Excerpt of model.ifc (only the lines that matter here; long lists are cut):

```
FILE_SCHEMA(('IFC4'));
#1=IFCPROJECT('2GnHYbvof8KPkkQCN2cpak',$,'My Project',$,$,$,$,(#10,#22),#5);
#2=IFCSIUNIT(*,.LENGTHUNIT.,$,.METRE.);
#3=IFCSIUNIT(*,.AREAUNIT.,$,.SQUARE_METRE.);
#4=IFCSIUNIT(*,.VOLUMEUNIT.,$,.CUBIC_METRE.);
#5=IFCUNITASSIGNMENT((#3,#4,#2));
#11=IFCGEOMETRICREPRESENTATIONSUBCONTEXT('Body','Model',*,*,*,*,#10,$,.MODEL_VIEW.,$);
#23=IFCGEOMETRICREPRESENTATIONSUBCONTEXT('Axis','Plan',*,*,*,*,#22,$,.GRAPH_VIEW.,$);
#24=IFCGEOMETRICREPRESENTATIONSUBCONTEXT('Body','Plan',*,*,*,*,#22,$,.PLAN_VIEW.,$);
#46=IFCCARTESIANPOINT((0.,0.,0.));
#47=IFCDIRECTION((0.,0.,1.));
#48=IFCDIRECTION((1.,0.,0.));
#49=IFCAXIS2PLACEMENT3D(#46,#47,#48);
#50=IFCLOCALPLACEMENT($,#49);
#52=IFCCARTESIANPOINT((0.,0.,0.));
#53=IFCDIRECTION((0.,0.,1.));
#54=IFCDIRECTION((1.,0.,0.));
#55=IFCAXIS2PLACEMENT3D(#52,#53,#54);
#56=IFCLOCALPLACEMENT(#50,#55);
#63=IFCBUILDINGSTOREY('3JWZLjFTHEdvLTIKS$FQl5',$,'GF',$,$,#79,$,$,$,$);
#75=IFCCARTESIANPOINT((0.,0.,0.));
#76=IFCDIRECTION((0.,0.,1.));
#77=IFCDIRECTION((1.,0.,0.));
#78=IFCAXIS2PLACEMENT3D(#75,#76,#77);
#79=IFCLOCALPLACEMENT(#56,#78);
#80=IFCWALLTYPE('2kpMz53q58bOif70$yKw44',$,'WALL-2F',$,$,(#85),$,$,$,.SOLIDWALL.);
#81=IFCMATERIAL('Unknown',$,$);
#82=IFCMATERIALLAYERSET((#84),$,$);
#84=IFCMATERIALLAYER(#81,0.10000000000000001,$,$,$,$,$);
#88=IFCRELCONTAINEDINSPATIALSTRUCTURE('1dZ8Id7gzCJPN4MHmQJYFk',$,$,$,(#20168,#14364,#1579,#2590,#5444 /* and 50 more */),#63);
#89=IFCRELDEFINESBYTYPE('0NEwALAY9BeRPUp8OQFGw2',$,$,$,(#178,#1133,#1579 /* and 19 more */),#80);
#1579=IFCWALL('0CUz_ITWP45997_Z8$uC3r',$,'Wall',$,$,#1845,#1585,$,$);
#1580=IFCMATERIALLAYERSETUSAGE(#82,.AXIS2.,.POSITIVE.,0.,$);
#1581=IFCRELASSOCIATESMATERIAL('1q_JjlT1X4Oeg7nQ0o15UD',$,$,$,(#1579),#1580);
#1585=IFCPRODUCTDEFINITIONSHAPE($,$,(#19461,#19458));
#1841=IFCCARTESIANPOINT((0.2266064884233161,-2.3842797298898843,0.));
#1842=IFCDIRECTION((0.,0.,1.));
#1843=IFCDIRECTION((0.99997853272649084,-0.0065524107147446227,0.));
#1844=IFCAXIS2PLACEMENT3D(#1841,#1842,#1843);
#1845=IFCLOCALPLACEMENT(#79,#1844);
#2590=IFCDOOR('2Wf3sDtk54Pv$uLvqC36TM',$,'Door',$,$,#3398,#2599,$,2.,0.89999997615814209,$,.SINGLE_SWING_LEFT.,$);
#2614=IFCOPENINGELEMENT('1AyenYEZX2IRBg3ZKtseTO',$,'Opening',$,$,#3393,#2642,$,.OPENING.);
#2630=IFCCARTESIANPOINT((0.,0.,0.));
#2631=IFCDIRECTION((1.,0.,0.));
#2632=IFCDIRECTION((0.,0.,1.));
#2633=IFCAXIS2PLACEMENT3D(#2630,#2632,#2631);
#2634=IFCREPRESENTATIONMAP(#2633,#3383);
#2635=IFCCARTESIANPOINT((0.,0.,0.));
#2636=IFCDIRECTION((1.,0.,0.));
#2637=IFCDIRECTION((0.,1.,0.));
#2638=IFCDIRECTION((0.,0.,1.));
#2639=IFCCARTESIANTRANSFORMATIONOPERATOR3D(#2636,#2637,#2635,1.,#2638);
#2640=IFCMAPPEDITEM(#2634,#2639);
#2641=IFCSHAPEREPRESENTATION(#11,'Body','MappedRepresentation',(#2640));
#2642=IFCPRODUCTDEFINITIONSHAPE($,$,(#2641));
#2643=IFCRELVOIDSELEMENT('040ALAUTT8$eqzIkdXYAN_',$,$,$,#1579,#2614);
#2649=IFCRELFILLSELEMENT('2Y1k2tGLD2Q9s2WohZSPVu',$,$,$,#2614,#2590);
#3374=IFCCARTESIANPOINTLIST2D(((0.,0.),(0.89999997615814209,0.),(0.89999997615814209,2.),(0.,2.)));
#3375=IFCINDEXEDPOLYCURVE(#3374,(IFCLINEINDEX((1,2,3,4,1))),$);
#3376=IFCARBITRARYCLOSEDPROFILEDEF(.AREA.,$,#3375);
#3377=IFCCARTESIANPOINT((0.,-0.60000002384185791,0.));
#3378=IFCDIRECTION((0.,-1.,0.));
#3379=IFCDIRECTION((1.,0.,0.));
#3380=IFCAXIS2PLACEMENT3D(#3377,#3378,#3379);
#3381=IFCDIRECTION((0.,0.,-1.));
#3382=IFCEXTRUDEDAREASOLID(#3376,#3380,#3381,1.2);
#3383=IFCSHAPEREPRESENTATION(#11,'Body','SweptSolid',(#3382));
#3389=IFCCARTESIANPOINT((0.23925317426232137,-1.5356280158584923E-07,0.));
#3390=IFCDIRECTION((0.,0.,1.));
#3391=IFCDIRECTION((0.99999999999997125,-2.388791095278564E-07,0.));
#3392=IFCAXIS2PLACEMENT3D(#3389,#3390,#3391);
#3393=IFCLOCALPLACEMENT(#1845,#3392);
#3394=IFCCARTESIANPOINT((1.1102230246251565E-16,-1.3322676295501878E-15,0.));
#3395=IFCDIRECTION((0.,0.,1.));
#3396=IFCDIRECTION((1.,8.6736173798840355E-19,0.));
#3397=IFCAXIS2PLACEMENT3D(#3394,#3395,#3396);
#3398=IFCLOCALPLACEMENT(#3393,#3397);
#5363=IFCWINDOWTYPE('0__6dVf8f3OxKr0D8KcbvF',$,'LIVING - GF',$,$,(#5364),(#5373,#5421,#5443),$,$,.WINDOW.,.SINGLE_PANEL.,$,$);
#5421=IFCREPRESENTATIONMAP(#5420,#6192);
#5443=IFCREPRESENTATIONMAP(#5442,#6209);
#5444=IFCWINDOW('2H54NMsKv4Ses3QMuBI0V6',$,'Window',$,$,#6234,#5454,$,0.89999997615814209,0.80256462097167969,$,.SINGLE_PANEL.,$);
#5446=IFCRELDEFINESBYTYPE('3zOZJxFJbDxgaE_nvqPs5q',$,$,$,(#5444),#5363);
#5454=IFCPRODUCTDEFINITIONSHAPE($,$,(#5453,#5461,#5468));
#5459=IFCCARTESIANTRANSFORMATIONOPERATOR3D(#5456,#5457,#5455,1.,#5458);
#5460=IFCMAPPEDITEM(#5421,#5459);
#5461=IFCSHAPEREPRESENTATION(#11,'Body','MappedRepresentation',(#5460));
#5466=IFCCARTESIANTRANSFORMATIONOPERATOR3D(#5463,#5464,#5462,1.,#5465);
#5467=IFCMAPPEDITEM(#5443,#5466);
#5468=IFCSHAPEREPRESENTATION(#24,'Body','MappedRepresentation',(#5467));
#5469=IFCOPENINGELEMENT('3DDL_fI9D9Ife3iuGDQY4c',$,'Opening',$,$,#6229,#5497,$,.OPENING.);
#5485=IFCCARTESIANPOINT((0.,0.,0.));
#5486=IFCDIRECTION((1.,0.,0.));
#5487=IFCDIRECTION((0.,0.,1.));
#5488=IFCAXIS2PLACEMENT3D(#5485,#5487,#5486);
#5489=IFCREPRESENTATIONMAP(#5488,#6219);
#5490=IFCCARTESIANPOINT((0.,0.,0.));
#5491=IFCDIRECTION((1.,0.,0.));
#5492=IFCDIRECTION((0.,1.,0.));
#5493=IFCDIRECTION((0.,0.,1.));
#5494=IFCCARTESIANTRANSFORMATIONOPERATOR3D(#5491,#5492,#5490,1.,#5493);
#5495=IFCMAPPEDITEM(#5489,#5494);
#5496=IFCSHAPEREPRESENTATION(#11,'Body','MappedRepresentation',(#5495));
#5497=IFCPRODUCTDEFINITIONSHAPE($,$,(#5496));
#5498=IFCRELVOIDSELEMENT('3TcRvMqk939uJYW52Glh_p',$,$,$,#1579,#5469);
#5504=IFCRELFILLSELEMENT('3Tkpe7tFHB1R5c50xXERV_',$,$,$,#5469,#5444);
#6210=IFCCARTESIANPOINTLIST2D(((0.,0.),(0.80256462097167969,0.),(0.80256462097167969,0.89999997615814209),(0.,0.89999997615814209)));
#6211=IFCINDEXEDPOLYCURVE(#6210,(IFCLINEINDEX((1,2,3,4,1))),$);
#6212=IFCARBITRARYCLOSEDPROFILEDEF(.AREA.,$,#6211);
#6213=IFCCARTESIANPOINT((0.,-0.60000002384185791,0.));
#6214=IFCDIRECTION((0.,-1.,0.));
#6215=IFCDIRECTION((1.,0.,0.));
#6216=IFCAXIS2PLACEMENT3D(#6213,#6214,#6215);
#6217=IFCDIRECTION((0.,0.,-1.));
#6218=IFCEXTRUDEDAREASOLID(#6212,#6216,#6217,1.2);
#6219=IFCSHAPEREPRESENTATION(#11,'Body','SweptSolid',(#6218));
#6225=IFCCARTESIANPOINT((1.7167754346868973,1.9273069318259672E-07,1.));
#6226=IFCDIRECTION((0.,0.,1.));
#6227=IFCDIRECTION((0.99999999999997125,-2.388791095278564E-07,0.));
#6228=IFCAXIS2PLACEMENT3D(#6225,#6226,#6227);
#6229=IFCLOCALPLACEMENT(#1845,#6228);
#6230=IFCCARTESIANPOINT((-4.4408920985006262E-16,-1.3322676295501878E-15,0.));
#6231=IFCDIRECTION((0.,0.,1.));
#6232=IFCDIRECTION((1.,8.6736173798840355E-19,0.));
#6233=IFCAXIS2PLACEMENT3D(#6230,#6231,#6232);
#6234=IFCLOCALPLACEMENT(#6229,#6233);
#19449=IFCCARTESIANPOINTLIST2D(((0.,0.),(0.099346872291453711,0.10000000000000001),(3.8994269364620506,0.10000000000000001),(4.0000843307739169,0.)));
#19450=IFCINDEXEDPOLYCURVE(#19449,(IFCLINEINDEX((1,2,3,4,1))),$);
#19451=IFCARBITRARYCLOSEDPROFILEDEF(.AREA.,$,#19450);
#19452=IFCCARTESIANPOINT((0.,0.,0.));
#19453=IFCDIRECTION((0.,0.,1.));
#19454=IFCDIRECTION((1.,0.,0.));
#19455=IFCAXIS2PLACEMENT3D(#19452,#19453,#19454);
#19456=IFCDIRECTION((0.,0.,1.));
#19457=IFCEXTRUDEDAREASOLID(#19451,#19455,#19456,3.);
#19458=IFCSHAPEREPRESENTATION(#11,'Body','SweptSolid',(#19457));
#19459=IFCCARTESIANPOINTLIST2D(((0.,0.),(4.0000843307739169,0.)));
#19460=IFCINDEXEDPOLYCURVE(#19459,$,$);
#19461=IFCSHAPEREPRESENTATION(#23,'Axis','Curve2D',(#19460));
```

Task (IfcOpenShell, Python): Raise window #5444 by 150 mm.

```python
import numpy as np
import ifcopenshell
import ifcopenshell.api.geometry
import ifcopenshell.util.placement
import ifcopenshell.util.unit

model = ifcopenshell.open("model.ifc")
unit_scale = ifcopenshell.util.unit.calculate_unit_scale(model)

window = model.by_id(5444)
opening = window.FillsVoids[0].RelatingOpeningElement
dz = 0.15

shift = np.array([0.0, 0.0, dz])
# The window is placed relative to its opening, so it follows when the opening moves.
matrix = ifcopenshell.util.placement.get_local_placement(opening.ObjectPlacement)
matrix[:3, 3] += shift
ifcopenshell.api.geometry.edit_object_placement(
    model, product=opening, matrix=matrix, is_si=False, should_transform_children=True
)

print(f"moved by {dz * unit_scale:+.3f} m")

model.write("model_edited.ifc")
```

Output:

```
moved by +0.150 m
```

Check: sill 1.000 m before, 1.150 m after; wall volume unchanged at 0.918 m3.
